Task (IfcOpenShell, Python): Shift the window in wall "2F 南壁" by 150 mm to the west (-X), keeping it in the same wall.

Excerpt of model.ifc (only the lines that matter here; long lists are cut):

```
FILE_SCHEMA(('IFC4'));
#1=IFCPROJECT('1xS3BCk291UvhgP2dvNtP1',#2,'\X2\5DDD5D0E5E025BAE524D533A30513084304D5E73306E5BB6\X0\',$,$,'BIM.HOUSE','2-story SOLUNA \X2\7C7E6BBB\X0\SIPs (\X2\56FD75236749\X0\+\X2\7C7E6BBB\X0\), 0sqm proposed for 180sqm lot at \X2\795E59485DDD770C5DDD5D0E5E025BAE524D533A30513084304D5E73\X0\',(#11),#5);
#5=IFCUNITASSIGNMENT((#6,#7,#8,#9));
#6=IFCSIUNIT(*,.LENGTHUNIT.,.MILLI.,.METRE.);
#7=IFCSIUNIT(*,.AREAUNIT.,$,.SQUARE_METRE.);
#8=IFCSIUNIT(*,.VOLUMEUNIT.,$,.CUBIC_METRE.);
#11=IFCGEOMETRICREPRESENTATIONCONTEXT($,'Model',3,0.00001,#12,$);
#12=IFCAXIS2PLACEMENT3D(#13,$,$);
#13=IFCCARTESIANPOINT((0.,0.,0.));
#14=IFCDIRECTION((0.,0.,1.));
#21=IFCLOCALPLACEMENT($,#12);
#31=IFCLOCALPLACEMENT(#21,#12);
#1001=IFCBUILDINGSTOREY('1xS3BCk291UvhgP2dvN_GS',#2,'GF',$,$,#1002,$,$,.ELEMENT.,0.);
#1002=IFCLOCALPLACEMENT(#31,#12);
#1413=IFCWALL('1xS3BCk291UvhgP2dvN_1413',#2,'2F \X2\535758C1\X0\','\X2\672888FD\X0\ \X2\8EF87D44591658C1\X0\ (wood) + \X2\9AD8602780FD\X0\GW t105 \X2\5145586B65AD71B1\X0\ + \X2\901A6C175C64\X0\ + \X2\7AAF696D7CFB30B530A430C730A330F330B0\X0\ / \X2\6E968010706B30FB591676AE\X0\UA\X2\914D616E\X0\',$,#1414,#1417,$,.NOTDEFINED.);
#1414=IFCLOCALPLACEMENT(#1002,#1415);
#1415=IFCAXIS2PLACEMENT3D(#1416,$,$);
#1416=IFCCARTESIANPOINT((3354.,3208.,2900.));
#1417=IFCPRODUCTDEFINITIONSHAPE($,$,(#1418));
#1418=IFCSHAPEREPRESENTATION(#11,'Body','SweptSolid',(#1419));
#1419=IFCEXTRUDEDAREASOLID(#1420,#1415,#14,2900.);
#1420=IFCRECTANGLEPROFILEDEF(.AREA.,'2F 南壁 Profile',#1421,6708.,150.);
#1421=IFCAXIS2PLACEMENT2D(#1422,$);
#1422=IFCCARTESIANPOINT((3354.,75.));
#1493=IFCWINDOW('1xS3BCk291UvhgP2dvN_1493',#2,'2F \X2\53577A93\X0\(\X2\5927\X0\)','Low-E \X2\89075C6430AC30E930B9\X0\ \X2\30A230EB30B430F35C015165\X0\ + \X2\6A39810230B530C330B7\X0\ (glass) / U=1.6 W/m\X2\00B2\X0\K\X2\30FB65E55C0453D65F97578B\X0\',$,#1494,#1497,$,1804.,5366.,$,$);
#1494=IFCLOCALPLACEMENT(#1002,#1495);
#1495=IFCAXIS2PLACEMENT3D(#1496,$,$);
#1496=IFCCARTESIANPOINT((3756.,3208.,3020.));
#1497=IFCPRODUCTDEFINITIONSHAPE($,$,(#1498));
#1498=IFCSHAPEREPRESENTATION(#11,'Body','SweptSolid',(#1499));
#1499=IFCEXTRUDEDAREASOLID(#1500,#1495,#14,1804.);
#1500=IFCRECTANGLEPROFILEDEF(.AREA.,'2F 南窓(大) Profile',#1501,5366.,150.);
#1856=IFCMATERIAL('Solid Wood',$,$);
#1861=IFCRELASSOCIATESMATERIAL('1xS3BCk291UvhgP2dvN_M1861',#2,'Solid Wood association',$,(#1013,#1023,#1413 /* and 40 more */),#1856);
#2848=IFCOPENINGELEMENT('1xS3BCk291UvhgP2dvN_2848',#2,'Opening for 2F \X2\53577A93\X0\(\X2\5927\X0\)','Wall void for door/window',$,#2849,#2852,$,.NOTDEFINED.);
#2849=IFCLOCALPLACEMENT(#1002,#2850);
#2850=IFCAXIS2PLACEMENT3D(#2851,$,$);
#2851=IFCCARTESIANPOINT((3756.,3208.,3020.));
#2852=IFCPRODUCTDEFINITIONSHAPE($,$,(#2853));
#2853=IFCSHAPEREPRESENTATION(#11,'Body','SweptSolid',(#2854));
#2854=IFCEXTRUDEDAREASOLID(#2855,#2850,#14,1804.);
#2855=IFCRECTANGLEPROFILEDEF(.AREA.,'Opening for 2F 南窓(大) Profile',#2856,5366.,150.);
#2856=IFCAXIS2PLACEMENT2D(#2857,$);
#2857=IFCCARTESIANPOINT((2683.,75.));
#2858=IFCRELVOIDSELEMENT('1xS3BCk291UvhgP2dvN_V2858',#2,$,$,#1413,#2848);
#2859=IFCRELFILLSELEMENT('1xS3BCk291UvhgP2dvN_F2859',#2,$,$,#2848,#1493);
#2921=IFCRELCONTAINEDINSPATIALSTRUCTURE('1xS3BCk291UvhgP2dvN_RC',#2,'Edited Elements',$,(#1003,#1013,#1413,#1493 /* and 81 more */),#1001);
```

```python
import ifcopenshell
import ifcopenshell.api.geometry
import ifcopenshell.util.placement
import ifcopenshell.util.unit

model = ifcopenshell.open("model.ifc")
unit_scale = ifcopenshell.util.unit.calculate_unit_scale(model)

window = model.by_guid("1xS3BCk291UvhgP2dvN_1493")
opening = window.FillsVoids[0].RelatingOpeningElement
wall = opening.VoidsElements[0].RelatingBuildingElement

wall_matrix = ifcopenshell.util.placement.get_local_placement(wall.ObjectPlacement)
shift = wall_matrix[:3, 0] * -0.15 / unit_scale
before = ifcopenshell.util.placement.get_local_placement(window.ObjectPlacement)[:3, 3].copy()

# The window is not placed relative to its opening, so move both.
for product in (opening, window):
    matrix = ifcopenshell.util.placement.get_local_placement(product.ObjectPlacement)
    matrix[:3, 3] += shift
    ifcopenshell.api.geometry.edit_object_placement(model, product=product, matrix=matrix, is_si=False)

after = ifcopenshell.util.placement.get_local_placement(window.ObjectPlacement)[:3, 3]
print("window moved by", (after - before).round(3) + 0.0)

model.write("model-out.ifc")
```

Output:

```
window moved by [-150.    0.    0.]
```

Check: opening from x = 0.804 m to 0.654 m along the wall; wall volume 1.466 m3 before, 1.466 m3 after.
